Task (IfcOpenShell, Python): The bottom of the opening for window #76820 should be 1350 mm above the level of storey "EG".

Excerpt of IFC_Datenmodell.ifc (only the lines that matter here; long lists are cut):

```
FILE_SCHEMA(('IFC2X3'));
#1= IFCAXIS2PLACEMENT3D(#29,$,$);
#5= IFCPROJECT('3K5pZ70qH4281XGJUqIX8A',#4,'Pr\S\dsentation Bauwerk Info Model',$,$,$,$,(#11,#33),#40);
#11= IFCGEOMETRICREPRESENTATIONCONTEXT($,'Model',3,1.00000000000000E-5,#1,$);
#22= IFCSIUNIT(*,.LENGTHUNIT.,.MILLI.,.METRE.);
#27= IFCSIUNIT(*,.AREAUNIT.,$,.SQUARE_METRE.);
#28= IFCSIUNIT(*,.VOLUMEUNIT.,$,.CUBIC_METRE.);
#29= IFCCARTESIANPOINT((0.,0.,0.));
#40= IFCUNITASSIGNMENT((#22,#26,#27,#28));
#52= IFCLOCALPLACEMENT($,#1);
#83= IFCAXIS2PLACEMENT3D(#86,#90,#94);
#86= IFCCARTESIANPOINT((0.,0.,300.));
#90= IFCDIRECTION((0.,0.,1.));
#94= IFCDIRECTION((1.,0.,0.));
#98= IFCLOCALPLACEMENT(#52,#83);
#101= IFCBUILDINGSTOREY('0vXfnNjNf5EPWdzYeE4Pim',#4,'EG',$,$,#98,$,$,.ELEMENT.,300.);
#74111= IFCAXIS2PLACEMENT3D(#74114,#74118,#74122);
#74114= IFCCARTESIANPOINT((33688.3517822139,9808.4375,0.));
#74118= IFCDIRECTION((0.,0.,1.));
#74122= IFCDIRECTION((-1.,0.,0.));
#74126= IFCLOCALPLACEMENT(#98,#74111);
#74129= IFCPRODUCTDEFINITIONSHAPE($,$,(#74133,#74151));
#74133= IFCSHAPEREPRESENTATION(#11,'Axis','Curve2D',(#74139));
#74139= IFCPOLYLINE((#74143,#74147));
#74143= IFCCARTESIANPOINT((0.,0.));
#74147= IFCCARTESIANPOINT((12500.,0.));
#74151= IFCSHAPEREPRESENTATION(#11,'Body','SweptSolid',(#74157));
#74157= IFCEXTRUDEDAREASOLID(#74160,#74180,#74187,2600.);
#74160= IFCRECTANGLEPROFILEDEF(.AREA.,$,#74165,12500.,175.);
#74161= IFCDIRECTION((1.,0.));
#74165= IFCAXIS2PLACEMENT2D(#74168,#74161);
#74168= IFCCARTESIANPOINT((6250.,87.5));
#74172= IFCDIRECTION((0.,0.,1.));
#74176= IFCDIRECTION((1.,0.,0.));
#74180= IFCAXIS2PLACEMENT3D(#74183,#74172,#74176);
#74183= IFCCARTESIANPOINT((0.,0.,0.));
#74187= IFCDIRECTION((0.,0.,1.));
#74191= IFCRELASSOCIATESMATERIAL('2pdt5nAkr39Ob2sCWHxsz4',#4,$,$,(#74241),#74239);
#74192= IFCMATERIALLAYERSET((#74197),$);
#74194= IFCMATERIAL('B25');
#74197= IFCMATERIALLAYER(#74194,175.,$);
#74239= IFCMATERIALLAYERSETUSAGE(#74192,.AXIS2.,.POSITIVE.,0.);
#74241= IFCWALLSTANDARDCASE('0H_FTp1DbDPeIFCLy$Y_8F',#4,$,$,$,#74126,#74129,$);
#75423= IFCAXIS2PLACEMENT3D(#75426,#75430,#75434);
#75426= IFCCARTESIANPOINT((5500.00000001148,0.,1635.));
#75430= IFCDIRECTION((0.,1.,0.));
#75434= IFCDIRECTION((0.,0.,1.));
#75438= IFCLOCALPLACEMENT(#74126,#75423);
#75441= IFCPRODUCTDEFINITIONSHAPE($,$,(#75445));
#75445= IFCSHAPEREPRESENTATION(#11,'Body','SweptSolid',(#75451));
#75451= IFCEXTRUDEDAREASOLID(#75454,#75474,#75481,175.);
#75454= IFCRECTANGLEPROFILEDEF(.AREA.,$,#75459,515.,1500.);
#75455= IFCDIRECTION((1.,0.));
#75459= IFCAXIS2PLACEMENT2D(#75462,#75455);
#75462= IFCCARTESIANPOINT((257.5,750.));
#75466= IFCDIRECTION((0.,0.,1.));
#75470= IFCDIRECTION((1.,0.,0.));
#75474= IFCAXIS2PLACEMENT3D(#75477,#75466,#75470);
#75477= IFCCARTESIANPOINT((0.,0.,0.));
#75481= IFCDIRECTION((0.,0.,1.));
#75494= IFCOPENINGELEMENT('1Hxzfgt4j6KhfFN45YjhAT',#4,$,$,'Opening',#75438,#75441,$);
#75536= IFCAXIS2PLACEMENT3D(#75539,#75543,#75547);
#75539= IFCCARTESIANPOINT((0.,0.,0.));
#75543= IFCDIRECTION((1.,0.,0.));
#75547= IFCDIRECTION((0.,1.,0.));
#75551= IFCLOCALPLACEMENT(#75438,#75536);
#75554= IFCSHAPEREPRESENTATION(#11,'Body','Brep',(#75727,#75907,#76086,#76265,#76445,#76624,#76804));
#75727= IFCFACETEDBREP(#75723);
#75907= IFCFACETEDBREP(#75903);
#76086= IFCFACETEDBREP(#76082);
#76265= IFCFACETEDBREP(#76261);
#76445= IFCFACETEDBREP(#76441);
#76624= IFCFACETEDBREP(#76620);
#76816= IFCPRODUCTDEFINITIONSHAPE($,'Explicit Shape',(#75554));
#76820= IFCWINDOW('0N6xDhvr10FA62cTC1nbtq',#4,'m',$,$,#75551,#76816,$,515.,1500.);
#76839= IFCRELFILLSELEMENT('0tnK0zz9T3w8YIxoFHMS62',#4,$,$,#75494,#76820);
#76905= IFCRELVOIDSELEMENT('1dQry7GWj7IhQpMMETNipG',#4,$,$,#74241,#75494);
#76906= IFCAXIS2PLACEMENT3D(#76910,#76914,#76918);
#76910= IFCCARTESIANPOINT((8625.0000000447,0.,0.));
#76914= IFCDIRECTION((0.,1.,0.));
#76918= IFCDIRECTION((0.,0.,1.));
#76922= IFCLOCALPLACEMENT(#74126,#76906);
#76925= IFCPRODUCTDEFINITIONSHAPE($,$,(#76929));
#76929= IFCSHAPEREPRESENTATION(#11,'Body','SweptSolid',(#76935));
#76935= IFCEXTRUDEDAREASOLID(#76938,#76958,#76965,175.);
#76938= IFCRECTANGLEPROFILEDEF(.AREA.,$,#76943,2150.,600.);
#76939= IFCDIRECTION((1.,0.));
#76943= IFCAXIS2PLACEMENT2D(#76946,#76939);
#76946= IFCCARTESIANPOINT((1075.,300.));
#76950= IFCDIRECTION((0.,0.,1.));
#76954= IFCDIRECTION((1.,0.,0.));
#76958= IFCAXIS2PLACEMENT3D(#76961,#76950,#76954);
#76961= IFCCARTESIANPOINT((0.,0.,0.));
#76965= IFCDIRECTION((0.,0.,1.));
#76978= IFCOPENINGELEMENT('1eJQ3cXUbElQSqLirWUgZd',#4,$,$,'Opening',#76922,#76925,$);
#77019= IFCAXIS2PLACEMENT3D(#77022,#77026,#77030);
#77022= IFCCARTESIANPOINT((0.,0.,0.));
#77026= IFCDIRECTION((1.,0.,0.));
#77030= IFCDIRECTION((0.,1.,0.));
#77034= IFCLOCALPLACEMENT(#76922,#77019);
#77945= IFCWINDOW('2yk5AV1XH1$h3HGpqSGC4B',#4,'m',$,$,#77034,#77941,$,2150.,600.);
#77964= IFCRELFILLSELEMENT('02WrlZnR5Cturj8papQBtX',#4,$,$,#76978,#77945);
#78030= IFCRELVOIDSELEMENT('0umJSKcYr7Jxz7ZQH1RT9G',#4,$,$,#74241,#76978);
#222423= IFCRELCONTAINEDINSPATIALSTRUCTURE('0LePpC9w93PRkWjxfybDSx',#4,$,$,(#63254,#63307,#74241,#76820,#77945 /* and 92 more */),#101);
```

```python
import numpy as np
import ifcopenshell
import ifcopenshell.api.geometry
import ifcopenshell.geom
import ifcopenshell.util.element
import ifcopenshell.util.placement
import ifcopenshell.util.shape
import ifcopenshell.util.unit

model = ifcopenshell.open("IFC_Datenmodell.ifc")
unit_scale = ifcopenshell.util.unit.calculate_unit_scale(model)

window = model.by_id(76820)
opening = window.FillsVoids[0].RelatingOpeningElement
storey = ifcopenshell.util.element.get_container(window, ifc_class="IfcBuildingStorey")
level = ifcopenshell.util.placement.get_local_placement(storey.ObjectPlacement)[2, 3]

# The opening's origin need not be at the sill, so measure its lowest point.
shape = ifcopenshell.geom.create_shape(ifcopenshell.geom.settings(), opening)
bottom = ifcopenshell.util.shape.get_shape_bottom_elevation(shape, shape.geometry) / unit_scale
dz = level + 1350.0 - bottom

shift = np.array([0.0, 0.0, dz])
# The window is placed relative to its opening, so it follows when the opening moves.
matrix = ifcopenshell.util.placement.get_local_placement(opening.ObjectPlacement)
matrix[:3, 3] += shift
ifcopenshell.api.geometry.edit_object_placement(
    model, product=opening, matrix=matrix, is_si=False, should_transform_children=True
)

print(f"moved by {dz * unit_scale:+.3f} m")

model.write("IFC_Datenmodell_updated.ifc")
```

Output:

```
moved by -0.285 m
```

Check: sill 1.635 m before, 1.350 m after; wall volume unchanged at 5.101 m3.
